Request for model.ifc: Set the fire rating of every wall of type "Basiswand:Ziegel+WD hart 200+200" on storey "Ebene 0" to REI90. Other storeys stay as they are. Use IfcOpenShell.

First a look at what the model holds.

```python
import ifcopenshell
import ifcopenshell.util.element

model = ifcopenshell.open("model.ifc")
print(model.schema)
storey = next(s for s in model.by_type("IfcBuildingStorey") if s.Name == "Ebene 0")
walls = [e for e in ifcopenshell.util.element.get_decomposition(storey) if e.is_a("IfcWall")]
seen = {}
for e in walls:
    element_type = ifcopenshell.util.element.get_type(e)
    key = (element_type.Name if element_type != e and element_type else None, ifcopenshell.util.element.get_pset(e, "Pset_WallCommon", "FireRating"))
    seen[key] = seen.get(key, 0) + 1
for (name, value), count in sorted(seen.items(), key=str):
    print(count, "x", name, "|", value)
```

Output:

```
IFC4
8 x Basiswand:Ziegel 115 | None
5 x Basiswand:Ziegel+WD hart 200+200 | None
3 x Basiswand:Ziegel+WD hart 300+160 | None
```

```python
import ifcopenshell
import ifcopenshell.api.pset
import ifcopenshell.util.element

model = ifcopenshell.open("model.ifc")

storey = next(s for s in model.by_type("IfcBuildingStorey") if s.Name == "Ebene 0")
walls = [e for e in ifcopenshell.util.element.get_decomposition(storey) if e.is_a("IfcWall")]

count = 0
for e in walls:
    element_type = ifcopenshell.util.element.get_type(e)
    if element_type in (None, e) or element_type.Name != "Basiswand:Ziegel+WD hart 200+200":
        continue
    # add_pset returns the element's existing set when there is one.
    pset = ifcopenshell.api.pset.add_pset(model, product=e, name="Pset_WallCommon")
    ifcopenshell.api.pset.edit_pset(model, pset=pset, properties={"FireRating": "REI90"})
    count += 1

print(count, "walls updated")

model.write("model_updated.ifc")
```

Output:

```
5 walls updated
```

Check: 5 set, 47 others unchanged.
